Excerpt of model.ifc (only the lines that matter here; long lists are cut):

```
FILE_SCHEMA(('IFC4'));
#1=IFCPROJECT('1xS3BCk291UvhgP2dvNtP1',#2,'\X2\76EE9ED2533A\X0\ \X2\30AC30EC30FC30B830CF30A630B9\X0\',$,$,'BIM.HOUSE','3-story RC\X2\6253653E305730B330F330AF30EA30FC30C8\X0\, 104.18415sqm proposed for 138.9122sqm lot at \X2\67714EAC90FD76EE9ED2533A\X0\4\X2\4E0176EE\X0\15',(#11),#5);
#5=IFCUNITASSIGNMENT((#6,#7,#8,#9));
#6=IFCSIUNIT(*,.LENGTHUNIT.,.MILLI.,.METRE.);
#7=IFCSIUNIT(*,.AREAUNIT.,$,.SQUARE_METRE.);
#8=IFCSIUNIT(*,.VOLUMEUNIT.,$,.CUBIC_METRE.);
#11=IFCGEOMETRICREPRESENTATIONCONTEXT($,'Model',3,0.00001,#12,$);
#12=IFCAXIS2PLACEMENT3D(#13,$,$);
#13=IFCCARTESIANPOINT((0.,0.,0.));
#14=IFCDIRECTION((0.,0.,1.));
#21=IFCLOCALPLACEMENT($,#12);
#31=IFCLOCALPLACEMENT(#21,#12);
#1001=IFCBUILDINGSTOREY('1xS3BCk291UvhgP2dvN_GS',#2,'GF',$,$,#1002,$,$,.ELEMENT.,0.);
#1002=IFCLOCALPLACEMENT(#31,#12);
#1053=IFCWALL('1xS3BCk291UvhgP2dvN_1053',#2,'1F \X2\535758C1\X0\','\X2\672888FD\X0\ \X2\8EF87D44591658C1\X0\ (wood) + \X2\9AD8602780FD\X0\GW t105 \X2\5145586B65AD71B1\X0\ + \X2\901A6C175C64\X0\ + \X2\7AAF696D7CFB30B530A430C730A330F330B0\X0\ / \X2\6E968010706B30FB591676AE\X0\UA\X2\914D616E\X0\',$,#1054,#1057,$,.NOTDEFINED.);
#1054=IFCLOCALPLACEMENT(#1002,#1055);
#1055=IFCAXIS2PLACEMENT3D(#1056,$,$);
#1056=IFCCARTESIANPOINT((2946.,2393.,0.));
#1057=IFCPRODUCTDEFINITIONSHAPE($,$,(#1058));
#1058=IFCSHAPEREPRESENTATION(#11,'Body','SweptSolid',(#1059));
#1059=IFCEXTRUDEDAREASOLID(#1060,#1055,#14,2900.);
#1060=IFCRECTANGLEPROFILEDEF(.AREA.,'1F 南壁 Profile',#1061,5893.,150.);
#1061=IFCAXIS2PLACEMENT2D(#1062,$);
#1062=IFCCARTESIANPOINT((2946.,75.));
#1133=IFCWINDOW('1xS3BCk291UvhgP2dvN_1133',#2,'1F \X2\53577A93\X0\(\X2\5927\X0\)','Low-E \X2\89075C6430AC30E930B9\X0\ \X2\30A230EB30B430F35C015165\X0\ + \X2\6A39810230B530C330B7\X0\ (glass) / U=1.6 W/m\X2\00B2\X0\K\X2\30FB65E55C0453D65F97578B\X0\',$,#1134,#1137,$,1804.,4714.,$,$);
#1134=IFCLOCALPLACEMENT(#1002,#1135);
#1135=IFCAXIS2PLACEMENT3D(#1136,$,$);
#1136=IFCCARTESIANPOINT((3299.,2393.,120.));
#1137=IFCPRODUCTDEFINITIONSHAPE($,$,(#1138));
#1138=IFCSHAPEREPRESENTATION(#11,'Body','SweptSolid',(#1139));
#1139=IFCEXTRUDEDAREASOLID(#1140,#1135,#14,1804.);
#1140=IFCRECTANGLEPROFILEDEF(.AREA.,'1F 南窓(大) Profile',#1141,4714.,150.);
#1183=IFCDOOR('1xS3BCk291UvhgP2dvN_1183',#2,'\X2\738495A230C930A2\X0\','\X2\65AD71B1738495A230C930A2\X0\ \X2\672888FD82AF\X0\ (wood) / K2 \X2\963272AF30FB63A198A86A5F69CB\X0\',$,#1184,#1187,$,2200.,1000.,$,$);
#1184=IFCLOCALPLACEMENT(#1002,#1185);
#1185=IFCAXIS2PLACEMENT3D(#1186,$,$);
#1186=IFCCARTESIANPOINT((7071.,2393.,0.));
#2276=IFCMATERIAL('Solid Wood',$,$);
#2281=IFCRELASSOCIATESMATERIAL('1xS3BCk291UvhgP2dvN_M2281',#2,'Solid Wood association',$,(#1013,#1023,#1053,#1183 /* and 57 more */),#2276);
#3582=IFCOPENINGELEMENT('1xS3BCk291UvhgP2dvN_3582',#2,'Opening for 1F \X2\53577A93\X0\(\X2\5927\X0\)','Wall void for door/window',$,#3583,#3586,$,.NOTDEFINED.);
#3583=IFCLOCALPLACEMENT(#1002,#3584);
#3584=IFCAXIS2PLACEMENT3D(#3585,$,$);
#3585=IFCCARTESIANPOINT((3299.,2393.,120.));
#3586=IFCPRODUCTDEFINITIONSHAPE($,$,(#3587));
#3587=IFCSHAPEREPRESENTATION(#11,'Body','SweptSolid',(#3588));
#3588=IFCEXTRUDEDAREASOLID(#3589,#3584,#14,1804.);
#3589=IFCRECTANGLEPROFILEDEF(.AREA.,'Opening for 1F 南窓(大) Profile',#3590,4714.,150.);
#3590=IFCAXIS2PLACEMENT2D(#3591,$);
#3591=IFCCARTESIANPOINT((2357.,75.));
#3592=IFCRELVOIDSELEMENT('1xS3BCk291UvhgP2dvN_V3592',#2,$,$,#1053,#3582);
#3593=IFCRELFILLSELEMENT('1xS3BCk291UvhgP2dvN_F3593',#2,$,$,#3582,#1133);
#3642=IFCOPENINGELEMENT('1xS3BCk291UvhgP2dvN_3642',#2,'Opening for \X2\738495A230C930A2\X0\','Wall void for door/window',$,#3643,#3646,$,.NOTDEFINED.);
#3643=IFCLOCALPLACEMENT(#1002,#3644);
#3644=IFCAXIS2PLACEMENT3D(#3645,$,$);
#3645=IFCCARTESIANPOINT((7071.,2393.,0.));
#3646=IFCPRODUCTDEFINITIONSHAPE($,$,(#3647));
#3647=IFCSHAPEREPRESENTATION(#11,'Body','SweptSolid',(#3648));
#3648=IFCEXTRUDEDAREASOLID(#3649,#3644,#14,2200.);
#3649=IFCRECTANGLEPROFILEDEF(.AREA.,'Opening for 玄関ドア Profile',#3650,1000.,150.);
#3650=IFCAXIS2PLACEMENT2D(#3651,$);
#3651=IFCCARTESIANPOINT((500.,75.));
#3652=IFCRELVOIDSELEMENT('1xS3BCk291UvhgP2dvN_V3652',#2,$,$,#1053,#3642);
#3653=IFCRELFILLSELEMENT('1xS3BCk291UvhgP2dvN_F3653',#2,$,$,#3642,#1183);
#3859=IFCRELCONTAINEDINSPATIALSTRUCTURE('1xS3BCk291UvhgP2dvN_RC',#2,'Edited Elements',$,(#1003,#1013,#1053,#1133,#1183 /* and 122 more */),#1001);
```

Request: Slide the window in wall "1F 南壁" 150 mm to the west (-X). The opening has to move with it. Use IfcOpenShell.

```python
import ifcopenshell
import ifcopenshell.api.geometry
import ifcopenshell.util.placement

model = ifcopenshell.open("model.ifc")

window = model.by_guid("1xS3BCk291UvhgP2dvN_1133")
opening = window.FillsVoids[0].RelatingOpeningElement
wall = opening.VoidsElements[0].RelatingBuildingElement

wall_matrix = ifcopenshell.util.placement.get_local_placement(wall.ObjectPlacement)
shift = wall_matrix[:3, 0] * -150.0
before = ifcopenshell.util.placement.get_local_placement(window.ObjectPlacement)[:3, 3].copy()

# The window is not placed relative to its opening, so move both.
for product in (opening, window):
    matrix = ifcopenshell.util.placement.get_local_placement(product.ObjectPlacement)
    matrix[:3, 3] += shift
    ifcopenshell.api.geometry.edit_object_placement(model, product=product, matrix=matrix, is_si=False)

after = ifcopenshell.util.placement.get_local_placement(window.ObjectPlacement)[:3, 3]
print("window moved by", (after - before).round(3) + 0.0)

model.write("model_rev.ifc")
```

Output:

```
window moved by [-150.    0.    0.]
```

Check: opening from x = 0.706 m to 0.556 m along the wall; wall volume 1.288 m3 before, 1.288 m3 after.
